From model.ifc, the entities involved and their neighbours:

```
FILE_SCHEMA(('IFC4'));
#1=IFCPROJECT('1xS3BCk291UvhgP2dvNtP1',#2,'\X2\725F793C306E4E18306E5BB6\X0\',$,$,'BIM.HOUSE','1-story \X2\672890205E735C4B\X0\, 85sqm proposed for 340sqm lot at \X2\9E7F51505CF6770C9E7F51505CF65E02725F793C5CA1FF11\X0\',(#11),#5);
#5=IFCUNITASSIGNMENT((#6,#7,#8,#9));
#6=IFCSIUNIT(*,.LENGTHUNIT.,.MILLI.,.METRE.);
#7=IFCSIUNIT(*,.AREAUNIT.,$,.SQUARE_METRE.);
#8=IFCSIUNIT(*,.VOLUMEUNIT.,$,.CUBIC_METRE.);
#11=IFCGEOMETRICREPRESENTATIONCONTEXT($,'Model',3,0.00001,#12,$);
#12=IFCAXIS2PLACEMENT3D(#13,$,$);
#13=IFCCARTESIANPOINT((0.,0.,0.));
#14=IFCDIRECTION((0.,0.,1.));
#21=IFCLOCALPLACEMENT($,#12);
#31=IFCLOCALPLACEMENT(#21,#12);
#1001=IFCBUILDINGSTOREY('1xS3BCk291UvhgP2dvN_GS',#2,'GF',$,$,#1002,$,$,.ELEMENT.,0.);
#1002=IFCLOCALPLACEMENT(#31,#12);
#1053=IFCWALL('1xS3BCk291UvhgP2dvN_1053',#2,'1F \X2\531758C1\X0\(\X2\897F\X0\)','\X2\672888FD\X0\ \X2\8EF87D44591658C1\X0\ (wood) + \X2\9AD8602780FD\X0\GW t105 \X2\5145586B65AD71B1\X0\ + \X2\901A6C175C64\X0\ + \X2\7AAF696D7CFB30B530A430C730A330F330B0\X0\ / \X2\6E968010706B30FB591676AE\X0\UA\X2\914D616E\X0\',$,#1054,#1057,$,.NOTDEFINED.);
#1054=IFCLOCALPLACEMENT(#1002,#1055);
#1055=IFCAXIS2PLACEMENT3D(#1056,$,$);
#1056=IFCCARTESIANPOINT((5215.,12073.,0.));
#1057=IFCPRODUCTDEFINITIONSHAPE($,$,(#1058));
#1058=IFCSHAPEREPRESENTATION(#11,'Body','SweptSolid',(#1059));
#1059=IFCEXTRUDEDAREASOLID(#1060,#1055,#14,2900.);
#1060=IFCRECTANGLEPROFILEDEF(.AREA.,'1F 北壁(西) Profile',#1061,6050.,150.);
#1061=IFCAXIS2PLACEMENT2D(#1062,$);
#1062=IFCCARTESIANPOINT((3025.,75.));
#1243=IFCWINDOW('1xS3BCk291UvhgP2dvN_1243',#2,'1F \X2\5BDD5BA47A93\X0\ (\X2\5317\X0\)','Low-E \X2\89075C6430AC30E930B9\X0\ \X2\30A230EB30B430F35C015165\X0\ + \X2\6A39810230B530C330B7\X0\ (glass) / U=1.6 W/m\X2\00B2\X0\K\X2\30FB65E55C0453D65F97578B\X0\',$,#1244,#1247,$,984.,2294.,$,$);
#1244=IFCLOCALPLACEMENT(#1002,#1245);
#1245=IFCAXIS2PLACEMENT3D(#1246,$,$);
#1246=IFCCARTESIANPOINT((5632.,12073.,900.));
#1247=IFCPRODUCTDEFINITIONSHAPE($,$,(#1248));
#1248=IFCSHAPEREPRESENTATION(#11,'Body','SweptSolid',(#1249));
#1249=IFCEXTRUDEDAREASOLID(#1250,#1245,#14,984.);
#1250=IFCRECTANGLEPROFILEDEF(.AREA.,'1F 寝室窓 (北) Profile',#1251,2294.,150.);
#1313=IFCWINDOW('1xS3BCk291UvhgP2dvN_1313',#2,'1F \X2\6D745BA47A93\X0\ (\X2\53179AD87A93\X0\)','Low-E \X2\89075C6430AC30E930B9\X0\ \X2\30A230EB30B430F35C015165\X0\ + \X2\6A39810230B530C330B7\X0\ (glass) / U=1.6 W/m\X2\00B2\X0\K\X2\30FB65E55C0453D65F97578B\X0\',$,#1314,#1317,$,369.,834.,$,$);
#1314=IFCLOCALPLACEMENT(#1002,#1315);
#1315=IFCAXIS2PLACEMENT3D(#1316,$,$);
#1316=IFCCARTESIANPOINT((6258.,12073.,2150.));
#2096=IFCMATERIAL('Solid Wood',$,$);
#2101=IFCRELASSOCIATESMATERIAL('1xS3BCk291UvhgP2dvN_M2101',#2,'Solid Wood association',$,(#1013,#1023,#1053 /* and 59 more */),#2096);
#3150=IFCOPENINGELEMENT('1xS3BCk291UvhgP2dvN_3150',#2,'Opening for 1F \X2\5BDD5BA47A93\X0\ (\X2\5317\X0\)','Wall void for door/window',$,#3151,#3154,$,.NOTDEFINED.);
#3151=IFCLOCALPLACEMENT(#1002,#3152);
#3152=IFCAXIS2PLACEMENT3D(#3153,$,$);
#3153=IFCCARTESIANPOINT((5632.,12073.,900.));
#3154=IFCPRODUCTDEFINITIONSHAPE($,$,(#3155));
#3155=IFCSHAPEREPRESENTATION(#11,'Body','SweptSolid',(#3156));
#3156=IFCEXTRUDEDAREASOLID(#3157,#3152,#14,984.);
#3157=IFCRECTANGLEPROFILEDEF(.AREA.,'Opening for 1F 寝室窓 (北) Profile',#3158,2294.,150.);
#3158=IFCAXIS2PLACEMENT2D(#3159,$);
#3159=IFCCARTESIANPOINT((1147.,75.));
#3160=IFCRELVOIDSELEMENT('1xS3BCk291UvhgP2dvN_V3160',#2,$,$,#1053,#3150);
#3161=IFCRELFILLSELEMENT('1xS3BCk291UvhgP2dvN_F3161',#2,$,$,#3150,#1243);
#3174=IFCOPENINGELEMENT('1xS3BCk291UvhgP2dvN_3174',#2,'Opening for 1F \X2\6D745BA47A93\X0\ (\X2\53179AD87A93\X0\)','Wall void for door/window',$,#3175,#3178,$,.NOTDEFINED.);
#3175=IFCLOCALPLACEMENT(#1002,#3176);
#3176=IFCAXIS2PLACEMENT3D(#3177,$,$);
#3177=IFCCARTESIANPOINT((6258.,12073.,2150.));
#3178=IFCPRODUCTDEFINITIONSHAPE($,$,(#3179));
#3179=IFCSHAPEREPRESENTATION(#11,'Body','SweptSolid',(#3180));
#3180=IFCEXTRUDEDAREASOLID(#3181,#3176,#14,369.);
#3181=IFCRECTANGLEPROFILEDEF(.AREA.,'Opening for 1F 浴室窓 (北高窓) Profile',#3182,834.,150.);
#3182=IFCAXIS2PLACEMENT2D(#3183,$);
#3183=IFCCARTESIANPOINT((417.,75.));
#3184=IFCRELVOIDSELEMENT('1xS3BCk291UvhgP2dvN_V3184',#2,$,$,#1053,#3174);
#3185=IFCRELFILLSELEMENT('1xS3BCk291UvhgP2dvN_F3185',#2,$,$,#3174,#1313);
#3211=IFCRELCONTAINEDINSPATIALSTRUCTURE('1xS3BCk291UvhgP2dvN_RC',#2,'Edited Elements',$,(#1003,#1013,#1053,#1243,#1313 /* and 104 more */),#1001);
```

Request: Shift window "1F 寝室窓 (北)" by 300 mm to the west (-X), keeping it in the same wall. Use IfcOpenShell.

```python
import ifcopenshell
import ifcopenshell.api.geometry
import ifcopenshell.util.placement
import ifcopenshell.util.unit

model = ifcopenshell.open("model.ifc")
unit_scale = ifcopenshell.util.unit.calculate_unit_scale(model)

window = model.by_id(1243)
opening = window.FillsVoids[0].RelatingOpeningElement
wall = opening.VoidsElements[0].RelatingBuildingElement

wall_matrix = ifcopenshell.util.placement.get_local_placement(wall.ObjectPlacement)
shift = wall_matrix[:3, 0] * -0.3 / unit_scale
before = ifcopenshell.util.placement.get_local_placement(window.ObjectPlacement)[:3, 3].copy()

# The window is not placed relative to its opening, so move both.
for product in (opening, window):
    matrix = ifcopenshell.util.placement.get_local_placement(product.ObjectPlacement)
    matrix[:3, 3] += shift
    ifcopenshell.api.geometry.edit_object_placement(model, product=product, matrix=matrix, is_si=False)

after = ifcopenshell.util.placement.get_local_placement(window.ObjectPlacement)[:3, 3]
print("window moved by", (after - before).round(3) + 0.0)

model.write("model-out.ifc")
```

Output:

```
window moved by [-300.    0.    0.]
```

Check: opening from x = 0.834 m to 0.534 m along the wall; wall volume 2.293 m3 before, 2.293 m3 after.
